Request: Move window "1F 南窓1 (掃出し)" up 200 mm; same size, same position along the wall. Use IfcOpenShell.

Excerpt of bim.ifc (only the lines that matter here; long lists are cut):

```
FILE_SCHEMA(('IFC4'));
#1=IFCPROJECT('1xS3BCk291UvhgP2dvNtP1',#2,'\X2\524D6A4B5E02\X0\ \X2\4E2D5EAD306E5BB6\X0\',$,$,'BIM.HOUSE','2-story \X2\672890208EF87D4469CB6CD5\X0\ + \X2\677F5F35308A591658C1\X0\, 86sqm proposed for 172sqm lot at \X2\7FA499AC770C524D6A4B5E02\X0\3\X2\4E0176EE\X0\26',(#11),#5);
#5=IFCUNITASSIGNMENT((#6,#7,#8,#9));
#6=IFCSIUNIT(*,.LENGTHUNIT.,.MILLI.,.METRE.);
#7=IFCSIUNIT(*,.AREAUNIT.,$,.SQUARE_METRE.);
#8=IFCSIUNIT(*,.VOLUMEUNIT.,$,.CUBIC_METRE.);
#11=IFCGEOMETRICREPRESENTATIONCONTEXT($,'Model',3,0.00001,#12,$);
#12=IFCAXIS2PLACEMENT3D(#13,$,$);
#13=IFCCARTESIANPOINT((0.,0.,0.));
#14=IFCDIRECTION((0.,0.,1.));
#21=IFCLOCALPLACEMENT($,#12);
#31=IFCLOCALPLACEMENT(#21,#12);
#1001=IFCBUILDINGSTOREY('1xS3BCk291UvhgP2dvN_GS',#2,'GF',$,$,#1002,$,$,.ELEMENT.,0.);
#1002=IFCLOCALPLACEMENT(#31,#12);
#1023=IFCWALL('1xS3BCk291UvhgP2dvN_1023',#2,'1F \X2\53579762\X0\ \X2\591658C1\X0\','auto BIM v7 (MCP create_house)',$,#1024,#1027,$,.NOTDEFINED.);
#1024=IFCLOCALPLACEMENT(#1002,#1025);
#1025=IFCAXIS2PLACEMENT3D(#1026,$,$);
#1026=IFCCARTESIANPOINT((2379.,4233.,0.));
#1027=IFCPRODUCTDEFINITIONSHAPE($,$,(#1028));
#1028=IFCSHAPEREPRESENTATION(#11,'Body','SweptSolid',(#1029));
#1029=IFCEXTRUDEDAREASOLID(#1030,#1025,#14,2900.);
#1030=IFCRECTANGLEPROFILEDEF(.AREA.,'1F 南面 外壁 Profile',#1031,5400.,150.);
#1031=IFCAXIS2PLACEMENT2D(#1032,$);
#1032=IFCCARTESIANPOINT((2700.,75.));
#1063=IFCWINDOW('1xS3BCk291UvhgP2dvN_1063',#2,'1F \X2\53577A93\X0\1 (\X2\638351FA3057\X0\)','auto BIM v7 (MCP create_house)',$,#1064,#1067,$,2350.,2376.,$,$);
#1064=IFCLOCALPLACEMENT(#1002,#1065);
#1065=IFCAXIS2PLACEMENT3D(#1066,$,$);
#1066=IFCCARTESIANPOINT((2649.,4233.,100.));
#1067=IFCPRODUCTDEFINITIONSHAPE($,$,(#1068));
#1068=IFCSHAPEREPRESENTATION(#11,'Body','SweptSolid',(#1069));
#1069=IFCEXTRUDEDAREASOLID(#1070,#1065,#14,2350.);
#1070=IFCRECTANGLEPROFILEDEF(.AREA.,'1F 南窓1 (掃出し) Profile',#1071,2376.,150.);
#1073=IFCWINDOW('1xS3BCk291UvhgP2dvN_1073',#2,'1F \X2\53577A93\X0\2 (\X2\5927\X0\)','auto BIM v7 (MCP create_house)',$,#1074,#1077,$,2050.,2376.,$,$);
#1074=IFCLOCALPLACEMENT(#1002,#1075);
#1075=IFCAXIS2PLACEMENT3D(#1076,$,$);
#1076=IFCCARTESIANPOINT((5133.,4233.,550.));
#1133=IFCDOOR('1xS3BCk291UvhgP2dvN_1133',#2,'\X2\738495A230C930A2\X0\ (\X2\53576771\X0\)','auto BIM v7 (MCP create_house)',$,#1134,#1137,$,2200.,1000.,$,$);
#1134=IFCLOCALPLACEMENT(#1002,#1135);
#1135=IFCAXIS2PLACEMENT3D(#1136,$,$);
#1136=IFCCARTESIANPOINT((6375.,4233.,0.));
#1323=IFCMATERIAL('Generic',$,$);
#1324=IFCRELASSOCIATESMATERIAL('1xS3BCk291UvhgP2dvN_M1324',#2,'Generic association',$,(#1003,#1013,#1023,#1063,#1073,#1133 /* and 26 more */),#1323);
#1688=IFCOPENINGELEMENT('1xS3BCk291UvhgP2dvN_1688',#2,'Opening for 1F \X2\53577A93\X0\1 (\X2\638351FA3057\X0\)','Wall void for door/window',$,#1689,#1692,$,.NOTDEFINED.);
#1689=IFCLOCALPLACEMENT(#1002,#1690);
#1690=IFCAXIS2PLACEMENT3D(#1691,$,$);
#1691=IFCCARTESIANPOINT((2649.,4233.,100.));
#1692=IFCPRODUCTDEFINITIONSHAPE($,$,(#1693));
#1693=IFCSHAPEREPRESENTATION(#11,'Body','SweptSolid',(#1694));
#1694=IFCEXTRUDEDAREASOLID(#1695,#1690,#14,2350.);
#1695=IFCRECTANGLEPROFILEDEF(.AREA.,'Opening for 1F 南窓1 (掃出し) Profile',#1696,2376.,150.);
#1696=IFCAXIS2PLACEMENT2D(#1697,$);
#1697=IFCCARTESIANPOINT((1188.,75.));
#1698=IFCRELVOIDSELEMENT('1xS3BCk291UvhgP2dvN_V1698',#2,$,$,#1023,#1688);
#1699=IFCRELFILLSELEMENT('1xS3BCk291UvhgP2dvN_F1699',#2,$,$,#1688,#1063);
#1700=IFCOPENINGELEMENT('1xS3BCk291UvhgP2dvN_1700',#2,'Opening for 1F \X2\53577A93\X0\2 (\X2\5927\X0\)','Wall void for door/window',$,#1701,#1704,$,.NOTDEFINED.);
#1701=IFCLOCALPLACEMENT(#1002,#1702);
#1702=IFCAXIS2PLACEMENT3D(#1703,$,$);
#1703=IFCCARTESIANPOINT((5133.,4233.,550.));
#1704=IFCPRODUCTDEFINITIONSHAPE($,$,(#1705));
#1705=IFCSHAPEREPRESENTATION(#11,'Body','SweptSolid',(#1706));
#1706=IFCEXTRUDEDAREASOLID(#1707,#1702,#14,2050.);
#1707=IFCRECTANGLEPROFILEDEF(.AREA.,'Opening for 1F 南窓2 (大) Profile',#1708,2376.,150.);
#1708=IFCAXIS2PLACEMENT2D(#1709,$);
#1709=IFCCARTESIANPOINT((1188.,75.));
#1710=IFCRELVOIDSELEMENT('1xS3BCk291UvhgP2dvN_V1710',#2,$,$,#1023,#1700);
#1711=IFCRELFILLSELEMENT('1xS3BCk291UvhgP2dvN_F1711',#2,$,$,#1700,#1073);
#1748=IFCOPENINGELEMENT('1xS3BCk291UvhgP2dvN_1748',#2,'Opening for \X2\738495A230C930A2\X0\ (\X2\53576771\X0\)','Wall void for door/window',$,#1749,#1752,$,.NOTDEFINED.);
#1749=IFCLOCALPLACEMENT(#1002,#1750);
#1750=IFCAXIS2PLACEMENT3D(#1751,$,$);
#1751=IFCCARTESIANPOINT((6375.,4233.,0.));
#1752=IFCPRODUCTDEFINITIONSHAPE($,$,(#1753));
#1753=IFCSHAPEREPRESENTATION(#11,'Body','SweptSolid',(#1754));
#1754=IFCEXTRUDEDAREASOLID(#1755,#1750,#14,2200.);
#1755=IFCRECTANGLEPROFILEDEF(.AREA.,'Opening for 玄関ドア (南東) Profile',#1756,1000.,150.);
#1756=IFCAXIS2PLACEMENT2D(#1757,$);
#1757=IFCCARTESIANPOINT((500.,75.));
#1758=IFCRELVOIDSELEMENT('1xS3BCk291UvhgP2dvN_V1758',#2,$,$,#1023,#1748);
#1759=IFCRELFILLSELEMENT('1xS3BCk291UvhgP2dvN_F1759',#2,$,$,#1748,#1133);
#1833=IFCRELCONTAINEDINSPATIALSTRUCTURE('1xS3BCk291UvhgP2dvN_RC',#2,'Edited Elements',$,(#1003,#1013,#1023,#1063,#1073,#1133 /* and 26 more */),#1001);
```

```python
import numpy as np
import ifcopenshell
import ifcopenshell.api.geometry
import ifcopenshell.util.placement
import ifcopenshell.util.unit

model = ifcopenshell.open("bim.ifc")
unit_scale = ifcopenshell.util.unit.calculate_unit_scale(model)

window = model.by_guid("1xS3BCk291UvhgP2dvN_1063")
opening = window.FillsVoids[0].RelatingOpeningElement
dz = 0.2 / unit_scale

shift = np.array([0.0, 0.0, dz])
# The window is not placed relative to its opening, so move both.
for product in (opening, window):
    matrix = ifcopenshell.util.placement.get_local_placement(product.ObjectPlacement)
    matrix[:3, 3] += shift
    ifcopenshell.api.geometry.edit_object_placement(model, product=product, matrix=matrix, is_si=False)

print(f"moved by {dz * unit_scale:+.3f} m")

model.write("bim_rev.ifc")
```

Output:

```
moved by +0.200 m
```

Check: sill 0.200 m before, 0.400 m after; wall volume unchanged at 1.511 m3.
